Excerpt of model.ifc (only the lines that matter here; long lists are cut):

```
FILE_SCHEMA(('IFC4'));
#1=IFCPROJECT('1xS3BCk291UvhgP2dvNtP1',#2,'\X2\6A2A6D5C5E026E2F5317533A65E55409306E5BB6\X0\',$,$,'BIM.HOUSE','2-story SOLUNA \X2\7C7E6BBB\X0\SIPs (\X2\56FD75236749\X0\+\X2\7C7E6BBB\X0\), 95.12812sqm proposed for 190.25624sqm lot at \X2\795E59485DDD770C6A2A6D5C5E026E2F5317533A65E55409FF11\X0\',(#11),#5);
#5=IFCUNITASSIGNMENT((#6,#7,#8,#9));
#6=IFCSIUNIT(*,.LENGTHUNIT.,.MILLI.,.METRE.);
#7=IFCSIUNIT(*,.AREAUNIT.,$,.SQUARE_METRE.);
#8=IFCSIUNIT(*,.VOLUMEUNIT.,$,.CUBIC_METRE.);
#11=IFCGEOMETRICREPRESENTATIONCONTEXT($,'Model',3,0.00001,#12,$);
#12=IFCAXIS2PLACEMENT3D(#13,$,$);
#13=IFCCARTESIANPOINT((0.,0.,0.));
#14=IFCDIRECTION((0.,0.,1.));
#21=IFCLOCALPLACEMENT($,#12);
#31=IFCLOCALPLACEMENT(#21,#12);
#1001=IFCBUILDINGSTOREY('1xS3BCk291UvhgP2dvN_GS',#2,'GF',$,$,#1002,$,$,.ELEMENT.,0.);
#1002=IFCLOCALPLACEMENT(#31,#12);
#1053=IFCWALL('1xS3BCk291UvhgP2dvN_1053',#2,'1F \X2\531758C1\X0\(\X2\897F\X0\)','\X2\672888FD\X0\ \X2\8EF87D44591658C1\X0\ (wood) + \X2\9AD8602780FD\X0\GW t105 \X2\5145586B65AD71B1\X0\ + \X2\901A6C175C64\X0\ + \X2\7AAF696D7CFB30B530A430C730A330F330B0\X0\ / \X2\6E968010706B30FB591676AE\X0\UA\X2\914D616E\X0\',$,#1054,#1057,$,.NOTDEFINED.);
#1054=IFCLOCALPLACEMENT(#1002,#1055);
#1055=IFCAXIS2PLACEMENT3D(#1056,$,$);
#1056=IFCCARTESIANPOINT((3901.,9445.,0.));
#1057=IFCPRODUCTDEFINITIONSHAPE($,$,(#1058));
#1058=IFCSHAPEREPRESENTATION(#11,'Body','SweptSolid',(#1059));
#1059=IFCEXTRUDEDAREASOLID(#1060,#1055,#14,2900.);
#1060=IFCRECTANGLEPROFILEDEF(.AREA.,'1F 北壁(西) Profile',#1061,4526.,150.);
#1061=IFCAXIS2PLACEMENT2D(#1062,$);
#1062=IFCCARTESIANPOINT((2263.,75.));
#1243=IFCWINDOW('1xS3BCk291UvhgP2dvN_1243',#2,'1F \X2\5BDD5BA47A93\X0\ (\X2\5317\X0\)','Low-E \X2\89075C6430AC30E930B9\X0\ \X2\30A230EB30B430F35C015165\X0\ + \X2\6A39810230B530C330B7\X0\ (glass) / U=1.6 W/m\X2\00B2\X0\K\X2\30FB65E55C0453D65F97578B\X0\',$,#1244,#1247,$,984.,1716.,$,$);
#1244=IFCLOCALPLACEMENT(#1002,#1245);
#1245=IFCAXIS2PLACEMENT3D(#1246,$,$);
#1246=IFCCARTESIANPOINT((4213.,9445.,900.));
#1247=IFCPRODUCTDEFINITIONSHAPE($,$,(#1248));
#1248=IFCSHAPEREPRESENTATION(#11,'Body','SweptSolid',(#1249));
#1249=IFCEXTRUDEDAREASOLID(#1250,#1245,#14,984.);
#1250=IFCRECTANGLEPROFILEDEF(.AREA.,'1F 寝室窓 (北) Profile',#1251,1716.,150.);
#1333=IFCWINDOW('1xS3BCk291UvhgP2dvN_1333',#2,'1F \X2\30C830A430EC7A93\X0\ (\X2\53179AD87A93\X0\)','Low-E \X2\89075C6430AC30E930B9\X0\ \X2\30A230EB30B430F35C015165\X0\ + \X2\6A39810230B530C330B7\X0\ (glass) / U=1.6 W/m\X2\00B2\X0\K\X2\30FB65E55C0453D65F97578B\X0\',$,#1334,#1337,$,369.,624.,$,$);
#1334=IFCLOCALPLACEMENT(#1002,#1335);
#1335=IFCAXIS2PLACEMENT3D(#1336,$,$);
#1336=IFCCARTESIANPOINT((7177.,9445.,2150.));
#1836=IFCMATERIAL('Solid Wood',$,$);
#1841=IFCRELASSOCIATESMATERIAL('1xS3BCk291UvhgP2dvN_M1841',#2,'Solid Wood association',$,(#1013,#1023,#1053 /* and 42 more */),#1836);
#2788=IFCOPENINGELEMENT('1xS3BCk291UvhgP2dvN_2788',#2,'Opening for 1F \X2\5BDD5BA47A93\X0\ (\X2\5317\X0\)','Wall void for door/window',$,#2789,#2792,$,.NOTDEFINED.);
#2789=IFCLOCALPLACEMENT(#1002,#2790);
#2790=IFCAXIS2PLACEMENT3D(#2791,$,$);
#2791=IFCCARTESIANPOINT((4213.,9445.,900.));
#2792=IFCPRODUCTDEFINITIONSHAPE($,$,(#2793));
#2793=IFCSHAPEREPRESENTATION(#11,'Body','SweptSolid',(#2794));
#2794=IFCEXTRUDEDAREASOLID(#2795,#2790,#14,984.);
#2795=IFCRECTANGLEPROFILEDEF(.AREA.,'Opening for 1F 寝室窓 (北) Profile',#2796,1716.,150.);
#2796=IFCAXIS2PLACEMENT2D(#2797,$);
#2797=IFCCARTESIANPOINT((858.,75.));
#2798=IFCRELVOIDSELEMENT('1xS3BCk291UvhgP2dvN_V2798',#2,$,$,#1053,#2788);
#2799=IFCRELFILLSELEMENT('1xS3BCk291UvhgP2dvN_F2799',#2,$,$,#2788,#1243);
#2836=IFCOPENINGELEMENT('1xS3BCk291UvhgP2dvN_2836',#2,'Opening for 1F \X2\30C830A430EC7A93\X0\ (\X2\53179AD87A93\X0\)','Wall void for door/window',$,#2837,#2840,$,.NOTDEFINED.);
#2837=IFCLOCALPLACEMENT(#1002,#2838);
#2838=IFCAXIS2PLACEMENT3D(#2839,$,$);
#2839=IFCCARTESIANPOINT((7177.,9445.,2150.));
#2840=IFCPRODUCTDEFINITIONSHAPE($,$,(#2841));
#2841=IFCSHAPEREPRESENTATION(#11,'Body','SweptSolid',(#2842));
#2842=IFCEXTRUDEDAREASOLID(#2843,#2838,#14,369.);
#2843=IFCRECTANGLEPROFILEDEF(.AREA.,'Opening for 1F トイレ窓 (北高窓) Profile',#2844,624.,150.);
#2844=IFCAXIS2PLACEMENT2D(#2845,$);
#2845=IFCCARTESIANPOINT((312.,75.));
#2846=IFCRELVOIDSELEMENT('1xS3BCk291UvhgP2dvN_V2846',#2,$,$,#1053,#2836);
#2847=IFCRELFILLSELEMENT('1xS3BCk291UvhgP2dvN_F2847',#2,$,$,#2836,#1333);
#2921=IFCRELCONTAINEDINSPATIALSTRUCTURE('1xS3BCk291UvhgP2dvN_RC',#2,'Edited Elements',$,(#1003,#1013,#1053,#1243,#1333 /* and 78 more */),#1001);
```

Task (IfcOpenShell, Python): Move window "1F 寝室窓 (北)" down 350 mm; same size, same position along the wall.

```python
import numpy as np
import ifcopenshell
import ifcopenshell.api.geometry
import ifcopenshell.util.placement
import ifcopenshell.util.unit

model = ifcopenshell.open("model.ifc")
unit_scale = ifcopenshell.util.unit.calculate_unit_scale(model)

window = model.by_guid("1xS3BCk291UvhgP2dvN_1243")
opening = window.FillsVoids[0].RelatingOpeningElement
dz = -350.0

shift = np.array([0.0, 0.0, dz])
# The window is not placed relative to its opening, so move both.
for product in (opening, window):
    matrix = ifcopenshell.util.placement.get_local_placement(product.ObjectPlacement)
    matrix[:3, 3] += shift
    ifcopenshell.api.geometry.edit_object_placement(model, product=product, matrix=matrix, is_si=False)

print(f"moved by {dz * unit_scale:+.3f} m")

model.write("model-out.ifc")
```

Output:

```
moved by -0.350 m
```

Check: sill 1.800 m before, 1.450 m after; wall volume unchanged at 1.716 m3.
